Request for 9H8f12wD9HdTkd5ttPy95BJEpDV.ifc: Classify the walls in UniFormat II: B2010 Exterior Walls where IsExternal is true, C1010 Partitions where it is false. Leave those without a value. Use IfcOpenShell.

First a look at what the model holds.

```python
import ifcopenshell
import ifcopenshell.util.element

model = ifcopenshell.open("9H8f12wD9HdTkd5ttPy95BJEpDV.ifc")
print(model.schema)
print("classifications:", [c.Name for c in model.by_type("IfcClassification")])
values = [ifcopenshell.util.element.get_pset(e, "Pset_WallCommon", "IsExternal") for e in model.by_type("IfcWall")]
for value in (True, False, None):
    print("IsExternal", value, values.count(value))
```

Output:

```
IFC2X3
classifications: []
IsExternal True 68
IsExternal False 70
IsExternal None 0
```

```python
import ifcopenshell
import ifcopenshell.api.classification
import ifcopenshell.util.element

model = ifcopenshell.open("9H8f12wD9HdTkd5ttPy95BJEpDV.ifc")

# IFC2X3 requires Source and Edition and has no link from the project to the system.
system = model.create_entity("IfcClassification", Source="ASTM", Edition="E1557", Name="UniFormat II")

walls = model.by_type("IfcWall")
external = {e: ifcopenshell.util.element.get_pset(e, "Pset_WallCommon", "IsExternal") for e in walls}
for flag, code, name in ((True, "B2010", "Exterior Walls"), (False, "C1010", "Partitions")):
    products = [e for e in walls if external[e] is flag]
    ifcopenshell.api.classification.add_reference(
        model, products=products, classification=system, identification=code, name=name
    )
    print(code, len(products))

model.write("9H8f12wD9HdTkd5ttPy95BJEpDV_v2.ifc")
```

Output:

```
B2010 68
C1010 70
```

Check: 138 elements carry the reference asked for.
